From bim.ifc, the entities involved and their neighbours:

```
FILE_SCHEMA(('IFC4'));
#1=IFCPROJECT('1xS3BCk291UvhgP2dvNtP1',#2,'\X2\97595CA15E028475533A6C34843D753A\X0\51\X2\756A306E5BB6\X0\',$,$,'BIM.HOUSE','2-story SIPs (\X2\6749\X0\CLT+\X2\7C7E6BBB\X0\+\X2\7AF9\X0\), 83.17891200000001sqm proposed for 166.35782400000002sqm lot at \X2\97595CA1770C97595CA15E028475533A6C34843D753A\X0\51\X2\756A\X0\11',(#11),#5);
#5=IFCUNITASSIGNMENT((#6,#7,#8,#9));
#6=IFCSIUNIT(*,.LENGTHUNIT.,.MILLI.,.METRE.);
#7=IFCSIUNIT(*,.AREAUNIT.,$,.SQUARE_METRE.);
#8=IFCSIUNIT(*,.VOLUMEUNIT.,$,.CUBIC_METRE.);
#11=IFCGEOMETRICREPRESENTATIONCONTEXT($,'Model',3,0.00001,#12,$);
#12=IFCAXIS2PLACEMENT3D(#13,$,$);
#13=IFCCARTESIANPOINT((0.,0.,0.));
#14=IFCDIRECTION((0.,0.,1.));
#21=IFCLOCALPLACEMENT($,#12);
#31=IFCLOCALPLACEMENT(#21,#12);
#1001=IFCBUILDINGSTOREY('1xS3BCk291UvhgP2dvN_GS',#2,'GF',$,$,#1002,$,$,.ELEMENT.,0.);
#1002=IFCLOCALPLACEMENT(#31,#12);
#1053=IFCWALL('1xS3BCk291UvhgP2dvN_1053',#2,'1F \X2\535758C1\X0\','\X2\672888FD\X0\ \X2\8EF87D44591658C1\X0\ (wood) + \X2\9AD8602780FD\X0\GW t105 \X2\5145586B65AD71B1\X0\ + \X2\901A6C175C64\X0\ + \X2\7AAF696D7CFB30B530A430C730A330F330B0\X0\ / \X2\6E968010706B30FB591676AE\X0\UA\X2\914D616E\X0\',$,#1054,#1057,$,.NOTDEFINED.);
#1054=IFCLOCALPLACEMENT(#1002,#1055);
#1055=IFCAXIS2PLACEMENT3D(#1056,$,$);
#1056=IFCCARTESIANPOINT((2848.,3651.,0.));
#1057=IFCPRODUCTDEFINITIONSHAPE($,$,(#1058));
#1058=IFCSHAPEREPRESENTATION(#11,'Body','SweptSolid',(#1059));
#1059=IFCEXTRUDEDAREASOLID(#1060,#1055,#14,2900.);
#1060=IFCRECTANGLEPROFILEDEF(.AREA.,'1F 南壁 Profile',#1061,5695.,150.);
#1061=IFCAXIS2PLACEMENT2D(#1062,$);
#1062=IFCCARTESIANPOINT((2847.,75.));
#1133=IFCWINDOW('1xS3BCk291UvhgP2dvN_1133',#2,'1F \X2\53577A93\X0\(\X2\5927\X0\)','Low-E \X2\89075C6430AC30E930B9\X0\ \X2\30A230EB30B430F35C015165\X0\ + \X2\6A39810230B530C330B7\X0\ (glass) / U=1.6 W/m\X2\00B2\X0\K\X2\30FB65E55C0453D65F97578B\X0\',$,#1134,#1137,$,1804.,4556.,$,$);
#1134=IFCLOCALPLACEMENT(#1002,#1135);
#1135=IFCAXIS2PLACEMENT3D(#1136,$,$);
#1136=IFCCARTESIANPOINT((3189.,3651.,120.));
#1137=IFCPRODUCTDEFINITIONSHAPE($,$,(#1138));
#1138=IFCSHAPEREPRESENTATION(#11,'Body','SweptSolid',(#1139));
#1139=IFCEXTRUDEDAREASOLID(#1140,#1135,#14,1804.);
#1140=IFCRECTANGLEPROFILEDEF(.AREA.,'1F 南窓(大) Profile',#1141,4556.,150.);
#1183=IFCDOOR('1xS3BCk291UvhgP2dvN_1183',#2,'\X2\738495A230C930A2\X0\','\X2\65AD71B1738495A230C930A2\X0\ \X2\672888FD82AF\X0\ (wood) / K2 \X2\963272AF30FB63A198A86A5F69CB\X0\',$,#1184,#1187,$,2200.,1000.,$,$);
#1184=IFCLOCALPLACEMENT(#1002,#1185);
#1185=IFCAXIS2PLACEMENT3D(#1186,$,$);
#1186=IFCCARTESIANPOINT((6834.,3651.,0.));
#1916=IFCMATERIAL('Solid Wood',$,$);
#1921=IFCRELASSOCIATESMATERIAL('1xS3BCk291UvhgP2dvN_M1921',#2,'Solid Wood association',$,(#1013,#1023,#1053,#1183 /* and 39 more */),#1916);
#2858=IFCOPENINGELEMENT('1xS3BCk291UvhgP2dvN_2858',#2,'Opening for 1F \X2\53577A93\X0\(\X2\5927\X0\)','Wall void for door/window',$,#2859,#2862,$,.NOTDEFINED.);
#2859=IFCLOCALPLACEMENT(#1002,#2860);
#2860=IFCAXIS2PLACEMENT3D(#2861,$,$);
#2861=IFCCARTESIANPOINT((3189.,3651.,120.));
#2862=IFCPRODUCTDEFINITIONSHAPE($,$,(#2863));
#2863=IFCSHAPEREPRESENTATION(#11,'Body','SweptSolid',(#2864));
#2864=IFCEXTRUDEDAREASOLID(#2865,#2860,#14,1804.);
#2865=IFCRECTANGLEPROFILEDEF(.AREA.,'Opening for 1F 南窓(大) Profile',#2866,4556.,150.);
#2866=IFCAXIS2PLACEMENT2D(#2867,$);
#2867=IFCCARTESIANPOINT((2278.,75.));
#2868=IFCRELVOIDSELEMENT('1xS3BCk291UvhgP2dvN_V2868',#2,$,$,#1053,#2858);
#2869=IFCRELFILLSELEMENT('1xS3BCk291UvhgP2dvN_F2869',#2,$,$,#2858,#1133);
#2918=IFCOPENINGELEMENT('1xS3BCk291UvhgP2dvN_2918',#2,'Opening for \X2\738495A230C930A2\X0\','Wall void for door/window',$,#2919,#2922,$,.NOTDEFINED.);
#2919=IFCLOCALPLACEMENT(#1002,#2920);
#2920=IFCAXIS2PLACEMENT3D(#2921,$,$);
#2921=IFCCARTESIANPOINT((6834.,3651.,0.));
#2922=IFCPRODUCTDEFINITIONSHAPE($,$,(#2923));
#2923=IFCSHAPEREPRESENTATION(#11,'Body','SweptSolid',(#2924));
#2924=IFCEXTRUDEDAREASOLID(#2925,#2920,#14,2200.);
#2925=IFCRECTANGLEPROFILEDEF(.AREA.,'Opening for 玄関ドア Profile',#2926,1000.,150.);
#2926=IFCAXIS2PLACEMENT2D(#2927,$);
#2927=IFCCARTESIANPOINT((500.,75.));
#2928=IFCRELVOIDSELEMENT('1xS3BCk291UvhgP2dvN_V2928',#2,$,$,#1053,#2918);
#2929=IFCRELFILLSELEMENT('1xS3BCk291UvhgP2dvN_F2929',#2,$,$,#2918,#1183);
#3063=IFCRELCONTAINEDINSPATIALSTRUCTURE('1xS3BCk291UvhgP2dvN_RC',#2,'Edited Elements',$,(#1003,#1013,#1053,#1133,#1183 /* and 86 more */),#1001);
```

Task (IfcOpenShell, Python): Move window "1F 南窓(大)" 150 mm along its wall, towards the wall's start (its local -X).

```python
import ifcopenshell
import ifcopenshell.api.geometry
import ifcopenshell.util.placement

model = ifcopenshell.open("bim.ifc")

window = model.by_guid("1xS3BCk291UvhgP2dvN_1133")
opening = window.FillsVoids[0].RelatingOpeningElement
wall = opening.VoidsElements[0].RelatingBuildingElement

wall_matrix = ifcopenshell.util.placement.get_local_placement(wall.ObjectPlacement)
shift = wall_matrix[:3, 0] * -150.0
before = ifcopenshell.util.placement.get_local_placement(window.ObjectPlacement)[:3, 3].copy()

# The window is not placed relative to its opening, so move both.
for product in (opening, window):
    matrix = ifcopenshell.util.placement.get_local_placement(product.ObjectPlacement)
    matrix[:3, 3] += shift
    ifcopenshell.api.geometry.edit_object_placement(model, product=product, matrix=matrix, is_si=False)

after = ifcopenshell.util.placement.get_local_placement(window.ObjectPlacement)[:3, 3]
print("window moved by", (after - before).round(3) + 0.0)

model.write("bim_updated.ifc")
```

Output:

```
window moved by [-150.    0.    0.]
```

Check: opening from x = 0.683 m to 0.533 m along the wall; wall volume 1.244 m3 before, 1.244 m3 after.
